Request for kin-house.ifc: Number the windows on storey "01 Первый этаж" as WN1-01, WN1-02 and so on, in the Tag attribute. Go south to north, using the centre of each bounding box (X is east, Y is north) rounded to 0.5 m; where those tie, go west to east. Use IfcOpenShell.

First a look at what the model holds.

```python
import ifcopenshell
import ifcopenshell.util.element
import ifcopenshell.util.placement

model = ifcopenshell.open("kin-house.ifc")
print(model.schema)
storey = next(s for s in model.by_type("IfcBuildingStorey") if s.Name == "01 Первый этаж")
windows = [e for e in ifcopenshell.util.element.get_decomposition(storey) if e.is_a("IfcWindow")]
for e in sorted(windows, key=lambda e: e.id()):
    origin = ifcopenshell.util.placement.get_local_placement(e.ObjectPlacement)[:3, 3]
    print(e.id(), e.Tag, e.Name, origin.round(2) + 0.0, sep=" | ")
```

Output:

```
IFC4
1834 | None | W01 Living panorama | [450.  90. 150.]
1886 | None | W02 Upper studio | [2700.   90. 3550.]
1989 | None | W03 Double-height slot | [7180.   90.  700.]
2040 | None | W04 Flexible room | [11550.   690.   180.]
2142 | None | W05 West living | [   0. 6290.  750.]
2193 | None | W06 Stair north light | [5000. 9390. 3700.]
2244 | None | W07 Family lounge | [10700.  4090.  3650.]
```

```python
import ifcopenshell
import ifcopenshell.geom
import ifcopenshell.util.element
import ifcopenshell.util.shape

model = ifcopenshell.open("kin-house.ifc")
settings = ifcopenshell.geom.settings()
settings.set("use-world-coords", True)


def centre(element):
    shape = ifcopenshell.geom.create_shape(settings, element)
    return ifcopenshell.util.shape.get_bbox_centroid(shape.geometry)


storey = next(s for s in model.by_type("IfcBuildingStorey") if s.Name == "01 Первый этаж")
windows = [e for e in ifcopenshell.util.element.get_decomposition(storey) if e.is_a("IfcWindow")]

# Insertion points can sit at a corner or the storey origin, so sort by the geometry (in metres).
centres = {e: centre(e) for e in windows}
windows.sort(key=lambda e: (round(centres[e][1] / 0.5), centres[e][0]))

for i, e in enumerate(windows, start=1):
    number = f"WN1-{i:02d}"
    e.Tag = number
    print(e.id(), number)

model.write("kin-house_rev.ifc")
```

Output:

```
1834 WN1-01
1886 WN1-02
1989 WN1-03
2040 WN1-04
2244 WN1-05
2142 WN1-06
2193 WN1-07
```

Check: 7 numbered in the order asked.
